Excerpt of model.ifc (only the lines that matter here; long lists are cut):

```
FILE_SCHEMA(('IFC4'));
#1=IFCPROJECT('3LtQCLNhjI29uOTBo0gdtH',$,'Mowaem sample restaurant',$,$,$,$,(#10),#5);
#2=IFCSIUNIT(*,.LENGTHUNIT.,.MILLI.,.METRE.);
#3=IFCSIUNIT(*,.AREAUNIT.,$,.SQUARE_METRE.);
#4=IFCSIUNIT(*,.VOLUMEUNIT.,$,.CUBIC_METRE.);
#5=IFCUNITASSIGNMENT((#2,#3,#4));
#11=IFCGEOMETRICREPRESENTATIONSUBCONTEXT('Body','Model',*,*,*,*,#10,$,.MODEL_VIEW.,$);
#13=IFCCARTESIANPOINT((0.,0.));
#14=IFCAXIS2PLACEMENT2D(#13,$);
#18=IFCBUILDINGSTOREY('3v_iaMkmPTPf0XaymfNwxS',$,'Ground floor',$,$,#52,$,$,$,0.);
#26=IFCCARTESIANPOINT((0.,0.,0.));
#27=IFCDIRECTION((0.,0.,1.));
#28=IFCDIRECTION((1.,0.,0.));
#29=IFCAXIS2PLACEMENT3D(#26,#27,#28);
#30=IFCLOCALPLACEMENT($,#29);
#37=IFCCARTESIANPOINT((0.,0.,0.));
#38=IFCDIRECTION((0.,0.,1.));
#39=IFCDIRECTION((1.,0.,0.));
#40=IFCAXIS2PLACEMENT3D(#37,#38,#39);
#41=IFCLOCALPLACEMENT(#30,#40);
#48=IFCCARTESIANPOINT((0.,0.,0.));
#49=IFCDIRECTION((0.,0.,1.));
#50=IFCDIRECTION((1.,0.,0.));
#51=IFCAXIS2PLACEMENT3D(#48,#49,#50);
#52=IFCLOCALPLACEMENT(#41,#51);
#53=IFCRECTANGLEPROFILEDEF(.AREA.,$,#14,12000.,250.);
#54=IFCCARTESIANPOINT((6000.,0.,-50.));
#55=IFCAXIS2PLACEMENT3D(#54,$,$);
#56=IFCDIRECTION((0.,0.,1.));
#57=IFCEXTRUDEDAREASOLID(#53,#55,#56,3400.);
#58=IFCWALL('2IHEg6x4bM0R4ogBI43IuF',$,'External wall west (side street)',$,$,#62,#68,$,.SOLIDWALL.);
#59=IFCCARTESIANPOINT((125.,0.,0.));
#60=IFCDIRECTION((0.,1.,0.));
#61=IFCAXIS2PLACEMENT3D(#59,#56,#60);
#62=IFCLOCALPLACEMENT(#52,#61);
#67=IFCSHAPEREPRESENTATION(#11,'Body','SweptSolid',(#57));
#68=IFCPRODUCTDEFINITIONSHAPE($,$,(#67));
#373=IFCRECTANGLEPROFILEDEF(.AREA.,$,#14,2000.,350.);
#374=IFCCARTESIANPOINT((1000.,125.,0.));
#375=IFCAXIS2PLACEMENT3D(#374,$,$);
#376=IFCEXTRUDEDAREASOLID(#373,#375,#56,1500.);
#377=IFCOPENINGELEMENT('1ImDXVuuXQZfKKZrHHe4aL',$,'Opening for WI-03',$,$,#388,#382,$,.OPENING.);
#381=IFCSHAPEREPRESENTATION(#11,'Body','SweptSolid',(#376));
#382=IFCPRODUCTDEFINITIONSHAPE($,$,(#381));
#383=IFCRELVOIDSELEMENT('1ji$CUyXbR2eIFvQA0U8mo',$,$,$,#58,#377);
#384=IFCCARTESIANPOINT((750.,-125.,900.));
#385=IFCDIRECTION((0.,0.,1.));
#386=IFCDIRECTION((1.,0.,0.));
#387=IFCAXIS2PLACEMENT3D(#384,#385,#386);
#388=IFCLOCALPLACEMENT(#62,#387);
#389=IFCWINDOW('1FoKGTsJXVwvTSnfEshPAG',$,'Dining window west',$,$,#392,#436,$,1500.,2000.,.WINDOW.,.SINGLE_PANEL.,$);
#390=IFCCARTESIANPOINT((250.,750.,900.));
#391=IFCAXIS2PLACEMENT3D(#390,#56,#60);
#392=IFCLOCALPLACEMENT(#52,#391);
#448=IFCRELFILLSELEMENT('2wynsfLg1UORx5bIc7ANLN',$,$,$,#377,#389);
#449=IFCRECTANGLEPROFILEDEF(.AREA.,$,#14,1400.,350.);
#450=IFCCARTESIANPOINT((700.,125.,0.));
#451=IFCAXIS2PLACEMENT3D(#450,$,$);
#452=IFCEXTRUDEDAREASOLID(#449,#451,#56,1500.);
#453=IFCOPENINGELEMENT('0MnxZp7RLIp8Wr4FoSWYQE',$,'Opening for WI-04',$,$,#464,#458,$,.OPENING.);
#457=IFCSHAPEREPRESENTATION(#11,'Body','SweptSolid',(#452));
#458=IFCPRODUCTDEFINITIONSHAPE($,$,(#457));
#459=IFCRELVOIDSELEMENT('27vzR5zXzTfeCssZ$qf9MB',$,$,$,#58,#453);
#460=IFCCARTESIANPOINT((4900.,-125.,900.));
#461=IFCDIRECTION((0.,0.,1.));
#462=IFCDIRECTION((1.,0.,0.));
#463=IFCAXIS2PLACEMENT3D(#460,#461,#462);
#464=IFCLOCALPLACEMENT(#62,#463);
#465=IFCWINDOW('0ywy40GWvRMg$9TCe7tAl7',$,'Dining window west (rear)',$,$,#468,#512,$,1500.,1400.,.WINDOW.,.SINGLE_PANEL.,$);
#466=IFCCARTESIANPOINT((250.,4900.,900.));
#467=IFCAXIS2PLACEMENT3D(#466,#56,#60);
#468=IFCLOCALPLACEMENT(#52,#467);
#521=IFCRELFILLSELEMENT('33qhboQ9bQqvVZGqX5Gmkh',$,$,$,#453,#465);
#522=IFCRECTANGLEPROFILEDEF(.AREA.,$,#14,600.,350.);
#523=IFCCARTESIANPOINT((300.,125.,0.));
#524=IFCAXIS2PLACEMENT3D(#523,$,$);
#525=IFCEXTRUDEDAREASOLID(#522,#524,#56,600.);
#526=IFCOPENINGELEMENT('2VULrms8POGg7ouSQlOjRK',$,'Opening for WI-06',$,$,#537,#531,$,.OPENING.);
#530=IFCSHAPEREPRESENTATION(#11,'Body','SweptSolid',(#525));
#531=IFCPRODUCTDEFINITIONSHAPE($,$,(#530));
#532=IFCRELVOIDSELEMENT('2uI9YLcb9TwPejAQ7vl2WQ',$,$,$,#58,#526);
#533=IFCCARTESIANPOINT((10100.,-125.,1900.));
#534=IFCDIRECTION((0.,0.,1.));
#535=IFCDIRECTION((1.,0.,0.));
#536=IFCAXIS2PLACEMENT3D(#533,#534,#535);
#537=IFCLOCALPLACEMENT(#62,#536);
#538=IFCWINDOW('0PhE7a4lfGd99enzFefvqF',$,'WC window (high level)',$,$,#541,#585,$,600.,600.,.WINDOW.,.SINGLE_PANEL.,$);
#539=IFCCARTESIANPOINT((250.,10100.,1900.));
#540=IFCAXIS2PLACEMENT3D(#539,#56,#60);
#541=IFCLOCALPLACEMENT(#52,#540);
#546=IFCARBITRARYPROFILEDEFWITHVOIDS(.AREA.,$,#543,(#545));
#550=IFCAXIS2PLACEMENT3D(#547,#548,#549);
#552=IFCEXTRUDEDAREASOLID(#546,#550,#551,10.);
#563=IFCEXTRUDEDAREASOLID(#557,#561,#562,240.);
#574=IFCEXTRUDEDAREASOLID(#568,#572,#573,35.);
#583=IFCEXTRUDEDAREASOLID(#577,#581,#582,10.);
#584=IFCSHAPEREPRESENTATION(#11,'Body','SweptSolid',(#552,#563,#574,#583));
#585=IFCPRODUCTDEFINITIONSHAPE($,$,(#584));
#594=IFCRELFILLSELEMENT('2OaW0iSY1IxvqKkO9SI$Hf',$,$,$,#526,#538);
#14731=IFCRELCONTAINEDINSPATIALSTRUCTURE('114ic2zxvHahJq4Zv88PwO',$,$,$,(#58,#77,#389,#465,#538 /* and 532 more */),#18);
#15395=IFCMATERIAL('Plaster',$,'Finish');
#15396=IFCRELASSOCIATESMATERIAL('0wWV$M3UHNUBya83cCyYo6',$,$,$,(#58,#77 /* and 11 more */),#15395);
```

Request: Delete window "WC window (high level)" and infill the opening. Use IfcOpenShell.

```python
import ifcopenshell
import ifcopenshell.api.feature
import ifcopenshell.api.root
import ifcopenshell.geom
import ifcopenshell.util.shape

model = ifcopenshell.open("model.ifc")
settings = ifcopenshell.geom.settings()


def volume(element):
    """Net volume in cubic metres, openings subtracted."""
    shape = ifcopenshell.geom.create_shape(settings, element)
    return ifcopenshell.util.shape.get_volume(shape.geometry)


window = model.by_guid("0PhE7a4lfGd99enzFefvqF")
opening = window.FillsVoids[0].RelatingOpeningElement
wall = opening.VoidsElements[0].RelatingBuildingElement
before = volume(wall)

ifcopenshell.api.root.remove_product(model, product=window)
ifcopenshell.api.feature.remove_feature(model, feature=opening)

after = volume(wall)

print(f"wall volume {before:.3f} -> {after:.3f} m3")

model.write("model_updated.ifc")
```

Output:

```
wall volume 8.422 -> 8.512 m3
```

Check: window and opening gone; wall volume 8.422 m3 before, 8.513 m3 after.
